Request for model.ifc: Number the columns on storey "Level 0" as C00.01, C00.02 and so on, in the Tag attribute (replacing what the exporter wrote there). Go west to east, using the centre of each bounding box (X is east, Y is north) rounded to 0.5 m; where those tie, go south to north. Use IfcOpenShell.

First a look at what the model holds.

```python
import ifcopenshell
import ifcopenshell.util.element
import ifcopenshell.util.placement

model = ifcopenshell.open("model.ifc")
print(model.schema)
storey = next(s for s in model.by_type("IfcBuildingStorey") if s.Name == "Level 0")
columns = [e for e in ifcopenshell.util.element.get_decomposition(storey) if e.is_a("IfcColumn")]
for e in sorted(columns, key=lambda e: e.id()):
    origin = ifcopenshell.util.placement.get_local_placement(e.ObjectPlacement)[:3, 3]
    print(e.id(), e.Tag, e.Name, origin.round(2) + 0.0, sep=" | ")
```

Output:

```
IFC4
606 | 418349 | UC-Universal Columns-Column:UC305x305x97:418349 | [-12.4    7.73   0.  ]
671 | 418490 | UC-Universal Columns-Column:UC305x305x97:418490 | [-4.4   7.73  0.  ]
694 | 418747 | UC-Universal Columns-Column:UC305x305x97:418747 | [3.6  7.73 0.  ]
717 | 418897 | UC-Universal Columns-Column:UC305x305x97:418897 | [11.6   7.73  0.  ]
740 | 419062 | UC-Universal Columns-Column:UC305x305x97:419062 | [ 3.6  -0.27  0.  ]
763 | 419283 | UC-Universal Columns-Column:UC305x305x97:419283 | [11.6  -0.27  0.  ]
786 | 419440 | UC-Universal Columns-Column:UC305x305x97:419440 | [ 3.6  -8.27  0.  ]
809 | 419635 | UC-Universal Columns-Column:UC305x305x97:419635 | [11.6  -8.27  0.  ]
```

```python
import ifcopenshell
import ifcopenshell.geom
import ifcopenshell.util.element
import ifcopenshell.util.shape

model = ifcopenshell.open("model.ifc")
settings = ifcopenshell.geom.settings()
settings.set("use-world-coords", True)


def centre(element):
    shape = ifcopenshell.geom.create_shape(settings, element)
    return ifcopenshell.util.shape.get_bbox_centroid(shape.geometry)


storey = next(s for s in model.by_type("IfcBuildingStorey") if s.Name == "Level 0")
columns = [e for e in ifcopenshell.util.element.get_decomposition(storey) if e.is_a("IfcColumn")]

# Insertion points can sit at a corner or the storey origin, so sort by the geometry (in metres).
centres = {e: centre(e) for e in columns}
columns.sort(key=lambda e: (round(centres[e][0] / 0.5), centres[e][1]))

for i, e in enumerate(columns, start=1):
    number = f"C00.{i:02d}"
    e.Tag = number
    print(e.id(), number)

model.write("model_v2.ifc")
```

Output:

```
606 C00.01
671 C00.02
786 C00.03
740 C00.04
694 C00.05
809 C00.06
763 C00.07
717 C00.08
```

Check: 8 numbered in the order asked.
